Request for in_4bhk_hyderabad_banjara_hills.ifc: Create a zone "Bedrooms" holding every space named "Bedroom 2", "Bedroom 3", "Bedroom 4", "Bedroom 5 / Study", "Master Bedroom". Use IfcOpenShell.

First a look at what the model holds.

```python
import ifcopenshell

model = ifcopenshell.open("in_4bhk_hyderabad_banjara_hills.ifc")
print(model.schema)
seen = {}
for space in model.by_type("IfcSpace"):
    seen[space.LongName] = seen.get(space.LongName, 0) + 1
for name, count in sorted(seen.items(), key=str):
    print(count, "x", name)
print("zones:", [z.Name for z in model.by_type("IfcZone")][:20])
```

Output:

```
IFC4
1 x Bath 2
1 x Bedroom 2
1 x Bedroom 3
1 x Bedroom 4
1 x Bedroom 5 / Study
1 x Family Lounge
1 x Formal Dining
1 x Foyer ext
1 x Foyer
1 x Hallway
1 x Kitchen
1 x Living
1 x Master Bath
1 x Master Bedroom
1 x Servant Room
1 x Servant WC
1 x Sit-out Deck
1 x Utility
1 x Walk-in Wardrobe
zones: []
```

```python
import ifcopenshell
import ifcopenshell.api.group
import ifcopenshell.api.root

model = ifcopenshell.open("in_4bhk_hyderabad_banjara_hills.ifc")

names = {"Bedroom 2", "Bedroom 3", "Bedroom 4", "Bedroom 5 / Study", "Master Bedroom"}
spaces = [s for s in model.by_type("IfcSpace") if s.LongName in names]

zone = ifcopenshell.api.root.create_entity(model, ifc_class="IfcZone", name="Bedrooms")
ifcopenshell.api.group.assign_group(model, products=spaces, group=zone)
print(len(spaces), "spaces in", zone.Name)

model.write("in_4bhk_hyderabad_banjara_hills_rev.ifc")
```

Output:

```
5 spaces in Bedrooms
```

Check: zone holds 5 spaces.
